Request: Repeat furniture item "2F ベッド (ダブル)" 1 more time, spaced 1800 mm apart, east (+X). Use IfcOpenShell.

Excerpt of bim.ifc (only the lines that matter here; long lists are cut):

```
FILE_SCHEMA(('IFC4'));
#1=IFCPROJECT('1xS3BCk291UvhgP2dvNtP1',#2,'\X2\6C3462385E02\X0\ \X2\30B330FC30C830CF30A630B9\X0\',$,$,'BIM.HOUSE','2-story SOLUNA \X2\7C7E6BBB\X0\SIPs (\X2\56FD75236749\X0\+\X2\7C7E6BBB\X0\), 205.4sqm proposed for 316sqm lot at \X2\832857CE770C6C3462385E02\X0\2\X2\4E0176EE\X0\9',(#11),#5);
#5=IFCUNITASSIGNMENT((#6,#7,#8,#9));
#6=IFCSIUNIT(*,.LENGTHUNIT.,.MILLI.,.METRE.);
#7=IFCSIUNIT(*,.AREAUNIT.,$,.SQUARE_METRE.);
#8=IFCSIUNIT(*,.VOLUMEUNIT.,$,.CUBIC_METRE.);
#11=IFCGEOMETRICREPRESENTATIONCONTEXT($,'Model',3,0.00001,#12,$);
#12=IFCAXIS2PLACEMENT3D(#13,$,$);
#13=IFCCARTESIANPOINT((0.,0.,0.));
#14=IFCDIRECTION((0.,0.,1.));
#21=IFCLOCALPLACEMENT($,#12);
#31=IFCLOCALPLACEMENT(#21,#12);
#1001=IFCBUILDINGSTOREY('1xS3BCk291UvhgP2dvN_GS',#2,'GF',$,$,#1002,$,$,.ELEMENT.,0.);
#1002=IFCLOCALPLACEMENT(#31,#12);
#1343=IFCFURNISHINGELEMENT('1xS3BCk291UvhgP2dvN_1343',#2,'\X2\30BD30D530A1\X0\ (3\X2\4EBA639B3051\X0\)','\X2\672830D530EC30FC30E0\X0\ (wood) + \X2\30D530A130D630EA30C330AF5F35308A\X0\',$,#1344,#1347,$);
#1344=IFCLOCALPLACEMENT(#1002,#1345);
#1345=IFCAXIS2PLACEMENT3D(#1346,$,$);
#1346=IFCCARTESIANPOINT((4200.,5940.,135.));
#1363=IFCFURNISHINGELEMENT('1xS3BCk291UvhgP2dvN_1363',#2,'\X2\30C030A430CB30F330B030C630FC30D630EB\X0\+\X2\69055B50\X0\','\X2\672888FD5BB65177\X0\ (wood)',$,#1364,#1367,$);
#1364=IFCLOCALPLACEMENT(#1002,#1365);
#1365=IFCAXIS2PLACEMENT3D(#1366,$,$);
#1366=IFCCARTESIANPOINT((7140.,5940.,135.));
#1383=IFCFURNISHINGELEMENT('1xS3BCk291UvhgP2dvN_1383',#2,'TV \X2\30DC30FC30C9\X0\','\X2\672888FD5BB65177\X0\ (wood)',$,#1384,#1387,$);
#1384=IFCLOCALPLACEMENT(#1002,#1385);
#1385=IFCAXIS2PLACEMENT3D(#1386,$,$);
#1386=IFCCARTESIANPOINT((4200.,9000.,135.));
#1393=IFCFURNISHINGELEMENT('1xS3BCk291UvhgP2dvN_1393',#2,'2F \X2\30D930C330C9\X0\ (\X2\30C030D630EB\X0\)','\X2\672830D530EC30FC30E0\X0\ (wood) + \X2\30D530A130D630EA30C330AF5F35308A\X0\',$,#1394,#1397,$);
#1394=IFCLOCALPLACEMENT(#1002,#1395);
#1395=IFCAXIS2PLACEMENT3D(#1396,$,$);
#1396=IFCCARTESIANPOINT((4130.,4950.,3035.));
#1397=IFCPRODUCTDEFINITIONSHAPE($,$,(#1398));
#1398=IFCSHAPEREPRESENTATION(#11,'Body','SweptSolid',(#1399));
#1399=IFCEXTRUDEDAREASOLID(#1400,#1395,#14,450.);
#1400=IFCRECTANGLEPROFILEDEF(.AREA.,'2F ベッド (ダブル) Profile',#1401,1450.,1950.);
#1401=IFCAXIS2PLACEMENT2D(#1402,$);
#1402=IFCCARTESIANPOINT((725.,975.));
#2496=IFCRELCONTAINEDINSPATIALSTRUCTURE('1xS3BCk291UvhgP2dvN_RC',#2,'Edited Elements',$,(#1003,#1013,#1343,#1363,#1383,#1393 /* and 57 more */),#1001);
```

```python
import numpy as np
import ifcopenshell
import ifcopenshell.api.geometry
import ifcopenshell.api.root
import ifcopenshell.util.element
import ifcopenshell.util.placement

model = ifcopenshell.open("bim.ifc")


def reuse_history(source, copy):
    """copy_class also copies each property set's owner history, people and application; keep the originals."""
    for rel in copy.IsDefinedBy:
        if rel.is_a("IfcRelDefinesByProperties") and (history := rel.RelatingPropertyDefinition.OwnerHistory):
            rel.RelatingPropertyDefinition.OwnerHistory = source.OwnerHistory
            ifcopenshell.util.element.remove_deep2(model, history)


source = model.by_guid("1xS3BCk291UvhgP2dvN_1393")
base = ifcopenshell.util.placement.get_local_placement(source.ObjectPlacement)
step = np.array([1.0, 0.0, 0.0]) * 1800.0

for i in range(1, 2):
    copy = ifcopenshell.api.root.copy_class(model, product=source)
    copy.Representation = ifcopenshell.util.element.copy_deep(
        model, source.Representation, exclude=["IfcGeometricRepresentationContext", "IfcRepresentationMap"]
    )
    reuse_history(source, copy)
    matrix = base.copy()
    matrix[:3, 3] += i * step
    print("added at", matrix[:3, 3].round(3) + 0.0)
    ifcopenshell.api.geometry.edit_object_placement(model, product=copy, matrix=matrix, is_si=False)

model.write("bim_updated.ifc")
```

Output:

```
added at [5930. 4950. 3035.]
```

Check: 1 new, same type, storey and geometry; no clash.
